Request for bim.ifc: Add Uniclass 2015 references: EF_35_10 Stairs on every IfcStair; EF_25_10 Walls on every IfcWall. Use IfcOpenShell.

First a look at what the model holds.

```python
import ifcopenshell

model = ifcopenshell.open("bim.ifc")
print(model.schema)
print("classifications:", [c.Name for c in model.by_type("IfcClassification")])
for ifc_class in ("IfcDoor", "IfcRoof", "IfcStair", "IfcWall", "IfcWindow"):
    print(ifc_class, len(model.by_type(ifc_class)))
```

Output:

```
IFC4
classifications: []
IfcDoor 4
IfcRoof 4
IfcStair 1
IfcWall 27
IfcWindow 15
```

```python
import ifcopenshell
import ifcopenshell.api.classification

model = ifcopenshell.open("bim.ifc")

system = ifcopenshell.api.classification.add_classification(model, classification="Uniclass 2015")

codes = {
    "IfcStair": ("EF_35_10", "Stairs"),
    "IfcWall": ("EF_25_10", "Walls"),
}
for ifc_class, (code, name) in codes.items():
    products = model.by_type(ifc_class)
    ifcopenshell.api.classification.add_reference(
        model, products=products, classification=system, identification=code, name=name
    )
    print(code, len(products))

model.write("bim_updated.ifc")
```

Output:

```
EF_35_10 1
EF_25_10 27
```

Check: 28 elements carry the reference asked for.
